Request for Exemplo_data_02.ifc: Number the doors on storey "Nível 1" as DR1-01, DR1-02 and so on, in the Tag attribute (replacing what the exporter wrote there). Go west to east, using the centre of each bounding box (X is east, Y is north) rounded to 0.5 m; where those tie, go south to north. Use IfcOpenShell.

First a look at what the model holds.

```python
import ifcopenshell
import ifcopenshell.util.element
import ifcopenshell.util.placement

model = ifcopenshell.open("Exemplo_data_02.ifc")
print(model.schema)
storey = next(s for s in model.by_type("IfcBuildingStorey") if s.Name == "Nível 1")
doors = [e for e in ifcopenshell.util.element.get_decomposition(storey) if e.is_a("IfcDoor")]
for e in sorted(doors, key=lambda e: e.id()):
    origin = ifcopenshell.util.placement.get_local_placement(e.ObjectPlacement)[:3, 3]
    print(e.id(), e.Tag, e.Name, origin.round(2) + 0.0, sep=" | ")
```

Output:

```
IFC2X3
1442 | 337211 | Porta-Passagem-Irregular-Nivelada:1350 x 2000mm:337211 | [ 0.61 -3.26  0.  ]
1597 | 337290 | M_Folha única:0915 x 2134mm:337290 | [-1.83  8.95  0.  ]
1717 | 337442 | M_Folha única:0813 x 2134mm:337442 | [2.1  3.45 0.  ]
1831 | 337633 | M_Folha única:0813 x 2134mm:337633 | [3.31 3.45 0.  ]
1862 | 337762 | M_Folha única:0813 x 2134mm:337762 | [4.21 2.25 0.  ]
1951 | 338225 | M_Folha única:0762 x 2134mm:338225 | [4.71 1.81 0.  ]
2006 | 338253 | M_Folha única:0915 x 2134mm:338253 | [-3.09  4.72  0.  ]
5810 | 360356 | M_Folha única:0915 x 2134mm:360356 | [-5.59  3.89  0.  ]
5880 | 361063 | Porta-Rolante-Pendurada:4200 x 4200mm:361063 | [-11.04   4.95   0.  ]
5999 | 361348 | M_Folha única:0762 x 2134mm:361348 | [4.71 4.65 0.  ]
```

```python
import ifcopenshell
import ifcopenshell.geom
import ifcopenshell.util.element
import ifcopenshell.util.shape

model = ifcopenshell.open("Exemplo_data_02.ifc")
settings = ifcopenshell.geom.settings()
settings.set("use-world-coords", True)


def centre(element):
    shape = ifcopenshell.geom.create_shape(settings, element)
    return ifcopenshell.util.shape.get_bbox_centroid(shape.geometry)


storey = next(s for s in model.by_type("IfcBuildingStorey") if s.Name == "Nível 1")
doors = [e for e in ifcopenshell.util.element.get_decomposition(storey) if e.is_a("IfcDoor")]

# Insertion points can sit at a corner or the storey origin, so sort by the geometry (in metres).
centres = {e: centre(e) for e in doors}
doors.sort(key=lambda e: (round(centres[e][0] / 0.5), centres[e][1]))

for i, e in enumerate(doors, start=1):
    number = f"DR1-{i:02d}"
    e.Tag = number
    print(e.id(), number)

model.write("Exemplo_data_02_rev.ifc")
```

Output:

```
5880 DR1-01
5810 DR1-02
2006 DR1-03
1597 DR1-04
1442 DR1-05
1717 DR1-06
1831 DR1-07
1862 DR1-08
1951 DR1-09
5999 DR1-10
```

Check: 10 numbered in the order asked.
